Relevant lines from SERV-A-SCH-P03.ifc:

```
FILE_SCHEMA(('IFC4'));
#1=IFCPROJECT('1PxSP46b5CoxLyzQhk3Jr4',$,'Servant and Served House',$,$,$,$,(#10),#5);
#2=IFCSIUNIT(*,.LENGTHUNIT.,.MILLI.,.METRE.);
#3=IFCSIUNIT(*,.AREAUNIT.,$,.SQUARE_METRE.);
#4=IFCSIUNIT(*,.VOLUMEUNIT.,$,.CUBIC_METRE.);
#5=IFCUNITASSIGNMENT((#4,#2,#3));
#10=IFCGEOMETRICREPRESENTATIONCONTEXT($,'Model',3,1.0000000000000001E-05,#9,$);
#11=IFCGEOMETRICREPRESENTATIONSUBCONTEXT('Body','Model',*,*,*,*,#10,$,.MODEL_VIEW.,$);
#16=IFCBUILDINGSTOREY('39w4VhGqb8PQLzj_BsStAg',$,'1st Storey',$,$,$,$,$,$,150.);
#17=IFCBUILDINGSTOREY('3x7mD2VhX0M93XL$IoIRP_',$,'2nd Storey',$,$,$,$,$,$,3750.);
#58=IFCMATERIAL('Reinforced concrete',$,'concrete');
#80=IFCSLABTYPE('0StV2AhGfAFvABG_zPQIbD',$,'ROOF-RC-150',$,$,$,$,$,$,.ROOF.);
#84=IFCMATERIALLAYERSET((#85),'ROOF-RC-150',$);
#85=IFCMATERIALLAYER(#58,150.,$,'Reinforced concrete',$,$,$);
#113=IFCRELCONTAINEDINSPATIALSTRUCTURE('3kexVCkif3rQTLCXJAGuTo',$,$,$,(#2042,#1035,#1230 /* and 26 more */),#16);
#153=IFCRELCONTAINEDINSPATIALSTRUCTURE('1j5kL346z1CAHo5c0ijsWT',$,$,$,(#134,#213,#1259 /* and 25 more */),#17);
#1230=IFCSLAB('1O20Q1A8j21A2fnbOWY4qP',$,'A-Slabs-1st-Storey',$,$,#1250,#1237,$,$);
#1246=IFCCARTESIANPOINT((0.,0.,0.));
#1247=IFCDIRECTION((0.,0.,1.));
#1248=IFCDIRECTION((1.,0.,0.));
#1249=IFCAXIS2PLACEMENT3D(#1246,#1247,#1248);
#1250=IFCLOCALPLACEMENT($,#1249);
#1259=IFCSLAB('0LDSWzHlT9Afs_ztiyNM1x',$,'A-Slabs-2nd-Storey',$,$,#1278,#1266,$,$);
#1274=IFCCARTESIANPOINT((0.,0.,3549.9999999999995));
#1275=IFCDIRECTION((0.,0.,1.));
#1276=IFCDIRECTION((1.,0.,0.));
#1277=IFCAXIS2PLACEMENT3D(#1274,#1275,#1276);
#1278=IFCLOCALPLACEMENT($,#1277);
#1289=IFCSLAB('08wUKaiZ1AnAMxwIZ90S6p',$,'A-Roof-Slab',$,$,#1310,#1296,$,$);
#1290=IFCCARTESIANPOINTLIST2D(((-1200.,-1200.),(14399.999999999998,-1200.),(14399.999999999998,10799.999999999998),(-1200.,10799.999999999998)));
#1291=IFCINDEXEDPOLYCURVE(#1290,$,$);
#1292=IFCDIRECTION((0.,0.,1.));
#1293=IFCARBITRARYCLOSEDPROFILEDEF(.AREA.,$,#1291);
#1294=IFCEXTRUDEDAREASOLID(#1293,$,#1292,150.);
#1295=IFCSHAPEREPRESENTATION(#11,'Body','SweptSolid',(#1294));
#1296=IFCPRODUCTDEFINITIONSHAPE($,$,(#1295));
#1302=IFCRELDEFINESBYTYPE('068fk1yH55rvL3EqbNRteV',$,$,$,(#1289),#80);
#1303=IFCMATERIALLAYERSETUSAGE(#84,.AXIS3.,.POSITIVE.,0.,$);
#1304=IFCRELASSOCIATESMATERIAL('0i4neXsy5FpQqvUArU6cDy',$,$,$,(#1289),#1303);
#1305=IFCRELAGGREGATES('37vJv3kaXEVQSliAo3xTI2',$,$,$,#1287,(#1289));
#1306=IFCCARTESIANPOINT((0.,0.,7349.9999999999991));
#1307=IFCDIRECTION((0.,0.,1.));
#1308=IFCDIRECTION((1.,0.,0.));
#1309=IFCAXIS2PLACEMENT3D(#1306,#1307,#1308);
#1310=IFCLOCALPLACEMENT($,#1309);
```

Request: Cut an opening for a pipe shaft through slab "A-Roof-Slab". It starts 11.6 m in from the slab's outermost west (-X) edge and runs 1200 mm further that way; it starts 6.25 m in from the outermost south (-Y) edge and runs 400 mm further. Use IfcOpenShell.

```python
import numpy as np
import ifcopenshell
import ifcopenshell.api.feature
import ifcopenshell.api.geometry
import ifcopenshell.api.root
import ifcopenshell.geom
import ifcopenshell.util.placement
import ifcopenshell.util.representation
import ifcopenshell.util.shape
import ifcopenshell.util.unit

model = ifcopenshell.open("SERV-A-SCH-P03.ifc")
unit_scale = ifcopenshell.util.unit.calculate_unit_scale(model)
settings = ifcopenshell.geom.settings()


def volume(element):
    """Net volume in cubic metres, openings subtracted."""
    shape = ifcopenshell.geom.create_shape(settings, element)
    return ifcopenshell.util.shape.get_volume(shape.geometry)


slab = model.by_id(1289)
before = volume(slab)

# Extent in the slab's own axes, in metres. The edges named are its -X and -Y sides.
slab_shape = ifcopenshell.geom.create_shape(settings, slab)
vertices = ifcopenshell.util.shape.get_vertices(slab_shape.geometry)
x_min, y_min, bottom = vertices.min(axis=0)
top = vertices[:, 2].max()

opening = ifcopenshell.api.root.create_entity(model, ifc_class="IfcOpeningElement", name="Pipe shaft opening", predefined_type="OPENING")
context = ifcopenshell.util.representation.get_context(model, "Model", "Body", "MODEL_VIEW")
width, depth = 1.2, 0.4
outline = [(0.0, 0.0), (width, 0.0), (width, depth), (0.0, depth), (0.0, 0.0)]
# Overshoot both faces by 50 mm so the cut is clean.
shape = ifcopenshell.api.geometry.add_slab_representation(
    model, context=context, depth=top - bottom + 0.1, polyline=outline
)
ifcopenshell.api.geometry.assign_representation(model, product=opening, representation=shape)

matrix = ifcopenshell.util.placement.get_local_placement(slab.ObjectPlacement)
matrix[:, 3] = matrix @ np.append(np.array([x_min + 11.6, y_min + 6.25, bottom - 0.05]) / unit_scale, 1.0)
ifcopenshell.api.geometry.edit_object_placement(model, product=opening, matrix=matrix, is_si=False)
ifcopenshell.api.feature.add_feature(model, feature=opening, element=slab)

after = volume(slab)

print(f"slab volume {before:.3f} -> {after:.3f} m3")

model.write("SERV-A-SCH-P03_rev.ifc")
```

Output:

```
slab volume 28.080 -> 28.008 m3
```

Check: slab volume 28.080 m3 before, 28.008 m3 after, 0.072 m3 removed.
